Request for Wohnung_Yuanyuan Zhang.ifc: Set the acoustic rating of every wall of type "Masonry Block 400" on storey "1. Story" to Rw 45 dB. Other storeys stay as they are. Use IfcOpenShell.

First a look at what the model holds.

```python
import ifcopenshell
import ifcopenshell.util.element

model = ifcopenshell.open("Wohnung_Yuanyuan Zhang.ifc")
print(model.schema)
storey = next(s for s in model.by_type("IfcBuildingStorey") if s.Name == "1. Story")
walls = [e for e in ifcopenshell.util.element.get_decomposition(storey) if e.is_a("IfcWall")]
seen = {}
for e in walls:
    element_type = ifcopenshell.util.element.get_type(e)
    key = (element_type.Name if element_type != e and element_type else None, ifcopenshell.util.element.get_pset(e, "Pset_WallCommon", "AcousticRating"))
    seen[key] = seen.get(key, 0) + 1
for (name, value), count in sorted(seen.items(), key=str):
    print(count, "x", name, "|", value)
```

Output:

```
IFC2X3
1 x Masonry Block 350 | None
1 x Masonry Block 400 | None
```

```python
import ifcopenshell
import ifcopenshell.api.pset
import ifcopenshell.util.element

model = ifcopenshell.open("Wohnung_Yuanyuan Zhang.ifc")

storey = next(s for s in model.by_type("IfcBuildingStorey") if s.Name == "1. Story")
walls = [e for e in ifcopenshell.util.element.get_decomposition(storey) if e.is_a("IfcWall")]

count = 0
for e in walls:
    element_type = ifcopenshell.util.element.get_type(e)
    if element_type in (None, e) or element_type.Name != "Masonry Block 400":
        continue
    # add_pset returns the element's existing set when there is one.
    pset = ifcopenshell.api.pset.add_pset(model, product=e, name="Pset_WallCommon")
    ifcopenshell.api.pset.edit_pset(model, pset=pset, properties={"AcousticRating": "Rw 45 dB"})
    count += 1

print(count, "walls updated")

model.write("Wohnung_Yuanyuan Zhang_edited.ifc")
```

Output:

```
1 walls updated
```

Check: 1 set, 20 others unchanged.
